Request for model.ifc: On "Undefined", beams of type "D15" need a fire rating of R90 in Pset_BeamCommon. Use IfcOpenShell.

First a look at what the model holds.

```python
import ifcopenshell
import ifcopenshell.util.element

model = ifcopenshell.open("model.ifc")
print(model.schema)
storey = next(s for s in model.by_type("IfcBuildingStorey") if s.Name == "Undefined")
beams = [e for e in ifcopenshell.util.element.get_decomposition(storey) if e.is_a("IfcBeam")]
seen = {}
for e in beams:
    element_type = ifcopenshell.util.element.get_type(e)
    key = (element_type.Name if element_type != e and element_type else None, ifcopenshell.util.element.get_pset(e, "Pset_BeamCommon", "FireRating"))
    seen[key] = seen.get(key, 0) + 1
for (name, value), count in sorted(seen.items(), key=str):
    print(count, "x", name, "|", value)
```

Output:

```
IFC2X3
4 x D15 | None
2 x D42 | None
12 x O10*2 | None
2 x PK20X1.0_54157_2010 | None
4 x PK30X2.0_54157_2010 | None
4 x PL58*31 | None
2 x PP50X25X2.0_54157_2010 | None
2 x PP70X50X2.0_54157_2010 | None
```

```python
import ifcopenshell
import ifcopenshell.api.pset
import ifcopenshell.util.element

model = ifcopenshell.open("model.ifc")

storey = next(s for s in model.by_type("IfcBuildingStorey") if s.Name == "Undefined")
beams = [e for e in ifcopenshell.util.element.get_decomposition(storey) if e.is_a("IfcBeam")]

count = 0
for e in beams:
    element_type = ifcopenshell.util.element.get_type(e)
    if element_type in (None, e) or element_type.Name != "D15":
        continue
    found = ifcopenshell.util.element.get_pset(e, "Pset_BeamCommon", should_inherit=False)
    if found:
        pset = model.by_id(found["id"])
        if len(ifcopenshell.util.element.get_elements_by_pset(pset)) > 1:
            pset = ifcopenshell.api.pset.unshare_pset(model, products=[e], pset=pset)[0]
    else:
        pset = ifcopenshell.api.pset.add_pset(model, product=e, name="Pset_BeamCommon")
    ifcopenshell.api.pset.edit_pset(model, pset=pset, properties={"FireRating": "R90"})
    count += 1

print(count, "beams updated")

model.write("model_v2.ifc")
```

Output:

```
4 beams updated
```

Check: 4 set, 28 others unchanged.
